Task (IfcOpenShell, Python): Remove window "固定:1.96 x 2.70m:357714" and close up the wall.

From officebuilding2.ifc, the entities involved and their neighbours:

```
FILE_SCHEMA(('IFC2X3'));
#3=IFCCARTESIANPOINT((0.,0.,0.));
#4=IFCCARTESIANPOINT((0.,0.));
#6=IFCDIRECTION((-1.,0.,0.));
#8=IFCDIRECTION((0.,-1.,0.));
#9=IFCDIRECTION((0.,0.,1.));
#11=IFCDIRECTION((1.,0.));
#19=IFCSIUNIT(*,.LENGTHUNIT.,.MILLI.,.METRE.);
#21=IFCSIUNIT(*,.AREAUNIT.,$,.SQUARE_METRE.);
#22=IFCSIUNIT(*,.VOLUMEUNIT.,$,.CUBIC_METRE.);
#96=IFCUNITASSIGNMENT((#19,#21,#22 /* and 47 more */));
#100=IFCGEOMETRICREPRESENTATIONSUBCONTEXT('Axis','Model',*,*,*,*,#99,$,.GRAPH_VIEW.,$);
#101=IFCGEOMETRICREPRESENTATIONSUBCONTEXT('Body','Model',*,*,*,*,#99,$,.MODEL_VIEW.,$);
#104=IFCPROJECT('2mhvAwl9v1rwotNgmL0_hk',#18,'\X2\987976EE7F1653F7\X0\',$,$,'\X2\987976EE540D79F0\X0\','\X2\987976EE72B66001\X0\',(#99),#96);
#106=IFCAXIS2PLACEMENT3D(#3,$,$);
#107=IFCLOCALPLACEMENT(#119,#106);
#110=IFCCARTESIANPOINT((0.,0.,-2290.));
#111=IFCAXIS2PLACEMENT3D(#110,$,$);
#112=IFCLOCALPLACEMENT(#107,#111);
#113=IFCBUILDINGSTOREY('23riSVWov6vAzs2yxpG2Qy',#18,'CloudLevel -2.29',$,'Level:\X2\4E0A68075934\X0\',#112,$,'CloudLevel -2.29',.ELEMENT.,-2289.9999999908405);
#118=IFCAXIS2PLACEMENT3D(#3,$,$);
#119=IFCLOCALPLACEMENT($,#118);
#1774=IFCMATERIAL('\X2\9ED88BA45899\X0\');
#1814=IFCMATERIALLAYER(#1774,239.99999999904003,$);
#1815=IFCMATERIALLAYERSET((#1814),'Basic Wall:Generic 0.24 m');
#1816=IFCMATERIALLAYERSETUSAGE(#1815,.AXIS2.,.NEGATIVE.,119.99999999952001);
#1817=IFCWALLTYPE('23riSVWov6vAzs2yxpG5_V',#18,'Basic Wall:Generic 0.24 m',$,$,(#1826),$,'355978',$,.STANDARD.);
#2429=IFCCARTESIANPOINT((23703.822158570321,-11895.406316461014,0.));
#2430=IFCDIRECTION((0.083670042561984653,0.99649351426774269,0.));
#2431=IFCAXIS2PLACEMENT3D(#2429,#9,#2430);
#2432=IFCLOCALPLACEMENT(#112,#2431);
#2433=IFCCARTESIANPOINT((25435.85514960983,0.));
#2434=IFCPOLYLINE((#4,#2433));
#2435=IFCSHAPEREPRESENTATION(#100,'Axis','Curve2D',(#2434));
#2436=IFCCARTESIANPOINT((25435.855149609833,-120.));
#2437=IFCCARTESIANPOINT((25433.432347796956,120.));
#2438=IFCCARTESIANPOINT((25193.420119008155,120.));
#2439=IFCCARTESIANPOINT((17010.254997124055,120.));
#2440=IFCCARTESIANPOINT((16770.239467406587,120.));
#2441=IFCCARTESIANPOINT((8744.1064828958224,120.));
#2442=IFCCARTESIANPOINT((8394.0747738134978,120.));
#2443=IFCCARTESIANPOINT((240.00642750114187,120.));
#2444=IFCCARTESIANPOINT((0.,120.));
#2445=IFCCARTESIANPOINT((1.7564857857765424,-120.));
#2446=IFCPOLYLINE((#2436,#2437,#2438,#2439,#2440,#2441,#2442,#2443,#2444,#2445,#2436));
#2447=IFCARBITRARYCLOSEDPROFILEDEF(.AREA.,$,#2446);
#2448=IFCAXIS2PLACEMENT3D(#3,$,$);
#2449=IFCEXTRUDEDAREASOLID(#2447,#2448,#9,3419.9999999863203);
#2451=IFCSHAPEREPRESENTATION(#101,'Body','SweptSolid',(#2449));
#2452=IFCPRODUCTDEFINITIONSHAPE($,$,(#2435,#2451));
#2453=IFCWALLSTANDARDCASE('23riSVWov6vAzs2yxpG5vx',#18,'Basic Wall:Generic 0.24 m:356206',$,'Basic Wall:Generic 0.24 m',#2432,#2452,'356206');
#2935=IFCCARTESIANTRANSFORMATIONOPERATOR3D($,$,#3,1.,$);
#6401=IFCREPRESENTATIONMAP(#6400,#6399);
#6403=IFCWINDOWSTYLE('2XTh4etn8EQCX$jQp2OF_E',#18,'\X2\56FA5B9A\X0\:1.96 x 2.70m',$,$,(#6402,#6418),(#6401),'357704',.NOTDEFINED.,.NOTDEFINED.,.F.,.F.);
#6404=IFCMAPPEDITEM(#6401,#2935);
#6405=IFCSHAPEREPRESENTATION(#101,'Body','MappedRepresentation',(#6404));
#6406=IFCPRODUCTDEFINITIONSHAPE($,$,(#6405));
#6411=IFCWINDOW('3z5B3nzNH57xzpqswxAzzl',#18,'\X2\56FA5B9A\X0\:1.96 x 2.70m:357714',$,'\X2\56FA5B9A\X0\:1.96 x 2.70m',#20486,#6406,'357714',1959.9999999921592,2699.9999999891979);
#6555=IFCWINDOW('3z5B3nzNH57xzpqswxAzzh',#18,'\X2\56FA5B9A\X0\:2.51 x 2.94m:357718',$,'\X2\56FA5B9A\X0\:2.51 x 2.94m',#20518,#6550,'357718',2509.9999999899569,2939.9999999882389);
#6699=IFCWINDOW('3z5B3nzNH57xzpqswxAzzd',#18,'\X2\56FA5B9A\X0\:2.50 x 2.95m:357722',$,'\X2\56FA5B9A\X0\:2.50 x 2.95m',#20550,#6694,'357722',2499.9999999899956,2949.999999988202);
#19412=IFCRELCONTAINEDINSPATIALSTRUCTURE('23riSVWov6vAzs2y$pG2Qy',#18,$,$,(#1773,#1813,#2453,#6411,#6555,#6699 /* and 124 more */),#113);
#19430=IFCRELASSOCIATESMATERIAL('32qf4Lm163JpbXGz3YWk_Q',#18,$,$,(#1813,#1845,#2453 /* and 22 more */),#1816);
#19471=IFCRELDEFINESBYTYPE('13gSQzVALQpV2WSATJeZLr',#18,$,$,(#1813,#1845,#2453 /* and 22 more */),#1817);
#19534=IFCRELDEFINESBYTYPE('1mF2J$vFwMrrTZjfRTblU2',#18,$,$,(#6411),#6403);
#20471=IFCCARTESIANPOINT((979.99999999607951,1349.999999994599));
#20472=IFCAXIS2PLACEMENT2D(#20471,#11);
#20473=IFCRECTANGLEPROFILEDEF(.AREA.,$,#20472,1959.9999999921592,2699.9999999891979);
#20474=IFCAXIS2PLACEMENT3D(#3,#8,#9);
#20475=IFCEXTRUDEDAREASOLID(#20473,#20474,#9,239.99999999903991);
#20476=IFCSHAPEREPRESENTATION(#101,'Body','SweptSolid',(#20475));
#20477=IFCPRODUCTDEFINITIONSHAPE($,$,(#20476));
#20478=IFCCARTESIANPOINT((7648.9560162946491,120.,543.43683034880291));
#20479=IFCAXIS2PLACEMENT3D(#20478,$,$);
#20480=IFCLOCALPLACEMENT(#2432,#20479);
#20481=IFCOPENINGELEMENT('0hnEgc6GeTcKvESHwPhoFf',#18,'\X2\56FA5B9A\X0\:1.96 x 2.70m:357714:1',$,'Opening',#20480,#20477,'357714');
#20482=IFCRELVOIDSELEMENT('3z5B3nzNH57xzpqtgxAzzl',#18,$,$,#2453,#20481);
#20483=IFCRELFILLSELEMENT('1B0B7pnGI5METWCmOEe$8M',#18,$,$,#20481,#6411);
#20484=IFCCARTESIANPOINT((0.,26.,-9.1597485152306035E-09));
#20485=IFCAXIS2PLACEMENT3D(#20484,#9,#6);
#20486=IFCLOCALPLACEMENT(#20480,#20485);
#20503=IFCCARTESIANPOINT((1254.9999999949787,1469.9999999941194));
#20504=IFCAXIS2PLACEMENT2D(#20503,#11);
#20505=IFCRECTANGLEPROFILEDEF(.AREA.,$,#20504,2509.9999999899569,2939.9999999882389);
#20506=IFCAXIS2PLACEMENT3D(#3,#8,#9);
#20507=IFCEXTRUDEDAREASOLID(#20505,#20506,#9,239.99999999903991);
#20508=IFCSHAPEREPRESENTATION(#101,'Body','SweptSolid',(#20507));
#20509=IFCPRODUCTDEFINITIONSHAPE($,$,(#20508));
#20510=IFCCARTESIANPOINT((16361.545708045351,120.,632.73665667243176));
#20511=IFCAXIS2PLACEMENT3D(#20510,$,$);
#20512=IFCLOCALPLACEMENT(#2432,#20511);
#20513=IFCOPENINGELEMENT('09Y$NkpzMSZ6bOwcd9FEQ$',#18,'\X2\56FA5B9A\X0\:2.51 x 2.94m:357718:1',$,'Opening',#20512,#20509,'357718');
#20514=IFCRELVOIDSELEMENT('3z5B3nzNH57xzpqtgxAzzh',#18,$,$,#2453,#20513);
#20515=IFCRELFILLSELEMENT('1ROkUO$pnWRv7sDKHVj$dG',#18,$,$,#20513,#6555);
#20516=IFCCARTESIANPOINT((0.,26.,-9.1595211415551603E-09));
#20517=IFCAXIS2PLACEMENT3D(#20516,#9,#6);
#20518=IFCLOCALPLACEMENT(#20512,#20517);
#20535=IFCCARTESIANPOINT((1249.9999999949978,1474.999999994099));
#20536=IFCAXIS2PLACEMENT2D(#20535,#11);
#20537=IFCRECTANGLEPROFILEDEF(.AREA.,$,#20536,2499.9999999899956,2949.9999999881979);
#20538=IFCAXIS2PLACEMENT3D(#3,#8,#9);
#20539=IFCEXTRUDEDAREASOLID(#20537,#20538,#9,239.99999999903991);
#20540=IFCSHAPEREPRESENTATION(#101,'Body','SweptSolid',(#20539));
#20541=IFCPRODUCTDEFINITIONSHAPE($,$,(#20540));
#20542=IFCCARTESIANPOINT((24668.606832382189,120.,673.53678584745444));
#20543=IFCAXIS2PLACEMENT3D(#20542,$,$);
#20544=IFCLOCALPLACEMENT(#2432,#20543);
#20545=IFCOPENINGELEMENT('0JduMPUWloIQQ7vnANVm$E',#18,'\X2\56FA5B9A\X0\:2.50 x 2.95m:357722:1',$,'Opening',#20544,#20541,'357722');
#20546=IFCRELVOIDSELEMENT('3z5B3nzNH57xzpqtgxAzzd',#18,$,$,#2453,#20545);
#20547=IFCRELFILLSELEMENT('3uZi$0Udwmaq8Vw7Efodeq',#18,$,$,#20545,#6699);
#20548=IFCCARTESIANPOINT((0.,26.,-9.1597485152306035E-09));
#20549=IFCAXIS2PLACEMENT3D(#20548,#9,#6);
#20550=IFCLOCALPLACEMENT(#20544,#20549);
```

```python
import ifcopenshell
import ifcopenshell.api.feature
import ifcopenshell.api.root
import ifcopenshell.geom
import ifcopenshell.util.shape

model = ifcopenshell.open("officebuilding2.ifc")
settings = ifcopenshell.geom.settings()


def volume(element):
    """Net volume in cubic metres, openings subtracted."""
    shape = ifcopenshell.geom.create_shape(settings, element)
    return ifcopenshell.util.shape.get_volume(shape.geometry)


window = model.by_id(6411)
opening = window.FillsVoids[0].RelatingOpeningElement
wall = opening.VoidsElements[0].RelatingBuildingElement
before = volume(wall)

ifcopenshell.api.root.remove_product(model, product=window)
ifcopenshell.api.feature.remove_feature(model, feature=opening)

after = volume(wall)

print(f"wall volume {before:.3f} -> {after:.3f} m3")

model.write("officebuilding2_updated.ifc")
```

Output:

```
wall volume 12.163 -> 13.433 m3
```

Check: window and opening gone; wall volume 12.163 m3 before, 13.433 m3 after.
